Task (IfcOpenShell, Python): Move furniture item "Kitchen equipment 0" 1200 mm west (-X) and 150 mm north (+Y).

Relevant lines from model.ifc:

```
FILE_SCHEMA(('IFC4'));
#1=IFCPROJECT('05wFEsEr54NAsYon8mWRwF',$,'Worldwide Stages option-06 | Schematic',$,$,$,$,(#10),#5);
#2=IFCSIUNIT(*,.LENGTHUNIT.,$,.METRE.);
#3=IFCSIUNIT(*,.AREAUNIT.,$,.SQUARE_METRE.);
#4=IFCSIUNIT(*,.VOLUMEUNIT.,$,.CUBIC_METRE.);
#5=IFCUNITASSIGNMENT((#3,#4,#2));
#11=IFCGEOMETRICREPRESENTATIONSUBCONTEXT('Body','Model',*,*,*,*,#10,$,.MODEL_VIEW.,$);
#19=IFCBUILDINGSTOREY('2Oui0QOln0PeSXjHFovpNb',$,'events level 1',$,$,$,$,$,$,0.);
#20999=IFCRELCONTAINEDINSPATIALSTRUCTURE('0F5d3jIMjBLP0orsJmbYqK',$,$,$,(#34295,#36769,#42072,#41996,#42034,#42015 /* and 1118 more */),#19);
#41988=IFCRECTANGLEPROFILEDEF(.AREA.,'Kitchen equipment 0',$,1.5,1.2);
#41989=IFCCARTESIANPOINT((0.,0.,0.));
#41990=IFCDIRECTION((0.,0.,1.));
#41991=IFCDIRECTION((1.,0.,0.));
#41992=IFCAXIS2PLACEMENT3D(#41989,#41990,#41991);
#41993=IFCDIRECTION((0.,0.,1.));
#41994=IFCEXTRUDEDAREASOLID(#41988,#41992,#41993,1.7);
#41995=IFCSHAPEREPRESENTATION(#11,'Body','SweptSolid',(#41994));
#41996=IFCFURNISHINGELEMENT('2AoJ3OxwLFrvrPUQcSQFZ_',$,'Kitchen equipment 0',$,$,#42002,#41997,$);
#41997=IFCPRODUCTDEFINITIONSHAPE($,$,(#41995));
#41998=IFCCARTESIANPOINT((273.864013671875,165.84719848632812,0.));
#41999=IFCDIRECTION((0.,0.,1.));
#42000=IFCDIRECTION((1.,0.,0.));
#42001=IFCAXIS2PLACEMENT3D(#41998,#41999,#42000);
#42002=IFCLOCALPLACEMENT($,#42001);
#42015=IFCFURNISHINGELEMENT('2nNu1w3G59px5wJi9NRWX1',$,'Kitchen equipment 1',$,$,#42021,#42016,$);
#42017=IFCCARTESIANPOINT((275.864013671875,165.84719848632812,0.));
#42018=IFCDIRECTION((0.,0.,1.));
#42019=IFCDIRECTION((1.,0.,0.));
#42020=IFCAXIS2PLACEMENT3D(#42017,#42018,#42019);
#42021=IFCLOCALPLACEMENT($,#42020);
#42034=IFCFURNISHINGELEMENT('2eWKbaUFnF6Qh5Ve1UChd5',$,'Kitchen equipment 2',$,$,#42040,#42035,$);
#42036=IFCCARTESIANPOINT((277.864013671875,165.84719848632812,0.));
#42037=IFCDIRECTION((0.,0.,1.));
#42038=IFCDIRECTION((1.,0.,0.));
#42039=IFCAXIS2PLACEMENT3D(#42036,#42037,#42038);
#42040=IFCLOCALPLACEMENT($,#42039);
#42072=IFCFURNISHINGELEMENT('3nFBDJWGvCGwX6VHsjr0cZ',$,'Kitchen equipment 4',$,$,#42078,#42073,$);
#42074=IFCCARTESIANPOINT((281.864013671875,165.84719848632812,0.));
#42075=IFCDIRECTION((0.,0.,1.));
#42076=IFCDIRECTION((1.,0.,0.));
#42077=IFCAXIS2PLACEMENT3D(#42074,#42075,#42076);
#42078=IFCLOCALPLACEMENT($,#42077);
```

```python
import ifcopenshell
import ifcopenshell.api.geometry
import ifcopenshell.util.placement
import ifcopenshell.util.unit

model = ifcopenshell.open("model.ifc")
unit_scale = ifcopenshell.util.unit.calculate_unit_scale(model)

item = model.by_guid("2AoJ3OxwLFrvrPUQcSQFZ_")
matrix = ifcopenshell.util.placement.get_local_placement(item.ObjectPlacement)
matrix[0, 3] -= 1.2 / unit_scale
matrix[1, 3] += 0.15 / unit_scale
ifcopenshell.api.geometry.edit_object_placement(model, product=item, matrix=matrix, is_si=False)

print(ifcopenshell.util.placement.get_local_placement(item.ObjectPlacement).round(3) + 0.0)

model.write("model_v2.ifc")
```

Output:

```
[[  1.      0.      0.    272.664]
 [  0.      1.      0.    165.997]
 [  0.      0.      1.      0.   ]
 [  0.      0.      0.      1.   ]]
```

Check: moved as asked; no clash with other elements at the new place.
